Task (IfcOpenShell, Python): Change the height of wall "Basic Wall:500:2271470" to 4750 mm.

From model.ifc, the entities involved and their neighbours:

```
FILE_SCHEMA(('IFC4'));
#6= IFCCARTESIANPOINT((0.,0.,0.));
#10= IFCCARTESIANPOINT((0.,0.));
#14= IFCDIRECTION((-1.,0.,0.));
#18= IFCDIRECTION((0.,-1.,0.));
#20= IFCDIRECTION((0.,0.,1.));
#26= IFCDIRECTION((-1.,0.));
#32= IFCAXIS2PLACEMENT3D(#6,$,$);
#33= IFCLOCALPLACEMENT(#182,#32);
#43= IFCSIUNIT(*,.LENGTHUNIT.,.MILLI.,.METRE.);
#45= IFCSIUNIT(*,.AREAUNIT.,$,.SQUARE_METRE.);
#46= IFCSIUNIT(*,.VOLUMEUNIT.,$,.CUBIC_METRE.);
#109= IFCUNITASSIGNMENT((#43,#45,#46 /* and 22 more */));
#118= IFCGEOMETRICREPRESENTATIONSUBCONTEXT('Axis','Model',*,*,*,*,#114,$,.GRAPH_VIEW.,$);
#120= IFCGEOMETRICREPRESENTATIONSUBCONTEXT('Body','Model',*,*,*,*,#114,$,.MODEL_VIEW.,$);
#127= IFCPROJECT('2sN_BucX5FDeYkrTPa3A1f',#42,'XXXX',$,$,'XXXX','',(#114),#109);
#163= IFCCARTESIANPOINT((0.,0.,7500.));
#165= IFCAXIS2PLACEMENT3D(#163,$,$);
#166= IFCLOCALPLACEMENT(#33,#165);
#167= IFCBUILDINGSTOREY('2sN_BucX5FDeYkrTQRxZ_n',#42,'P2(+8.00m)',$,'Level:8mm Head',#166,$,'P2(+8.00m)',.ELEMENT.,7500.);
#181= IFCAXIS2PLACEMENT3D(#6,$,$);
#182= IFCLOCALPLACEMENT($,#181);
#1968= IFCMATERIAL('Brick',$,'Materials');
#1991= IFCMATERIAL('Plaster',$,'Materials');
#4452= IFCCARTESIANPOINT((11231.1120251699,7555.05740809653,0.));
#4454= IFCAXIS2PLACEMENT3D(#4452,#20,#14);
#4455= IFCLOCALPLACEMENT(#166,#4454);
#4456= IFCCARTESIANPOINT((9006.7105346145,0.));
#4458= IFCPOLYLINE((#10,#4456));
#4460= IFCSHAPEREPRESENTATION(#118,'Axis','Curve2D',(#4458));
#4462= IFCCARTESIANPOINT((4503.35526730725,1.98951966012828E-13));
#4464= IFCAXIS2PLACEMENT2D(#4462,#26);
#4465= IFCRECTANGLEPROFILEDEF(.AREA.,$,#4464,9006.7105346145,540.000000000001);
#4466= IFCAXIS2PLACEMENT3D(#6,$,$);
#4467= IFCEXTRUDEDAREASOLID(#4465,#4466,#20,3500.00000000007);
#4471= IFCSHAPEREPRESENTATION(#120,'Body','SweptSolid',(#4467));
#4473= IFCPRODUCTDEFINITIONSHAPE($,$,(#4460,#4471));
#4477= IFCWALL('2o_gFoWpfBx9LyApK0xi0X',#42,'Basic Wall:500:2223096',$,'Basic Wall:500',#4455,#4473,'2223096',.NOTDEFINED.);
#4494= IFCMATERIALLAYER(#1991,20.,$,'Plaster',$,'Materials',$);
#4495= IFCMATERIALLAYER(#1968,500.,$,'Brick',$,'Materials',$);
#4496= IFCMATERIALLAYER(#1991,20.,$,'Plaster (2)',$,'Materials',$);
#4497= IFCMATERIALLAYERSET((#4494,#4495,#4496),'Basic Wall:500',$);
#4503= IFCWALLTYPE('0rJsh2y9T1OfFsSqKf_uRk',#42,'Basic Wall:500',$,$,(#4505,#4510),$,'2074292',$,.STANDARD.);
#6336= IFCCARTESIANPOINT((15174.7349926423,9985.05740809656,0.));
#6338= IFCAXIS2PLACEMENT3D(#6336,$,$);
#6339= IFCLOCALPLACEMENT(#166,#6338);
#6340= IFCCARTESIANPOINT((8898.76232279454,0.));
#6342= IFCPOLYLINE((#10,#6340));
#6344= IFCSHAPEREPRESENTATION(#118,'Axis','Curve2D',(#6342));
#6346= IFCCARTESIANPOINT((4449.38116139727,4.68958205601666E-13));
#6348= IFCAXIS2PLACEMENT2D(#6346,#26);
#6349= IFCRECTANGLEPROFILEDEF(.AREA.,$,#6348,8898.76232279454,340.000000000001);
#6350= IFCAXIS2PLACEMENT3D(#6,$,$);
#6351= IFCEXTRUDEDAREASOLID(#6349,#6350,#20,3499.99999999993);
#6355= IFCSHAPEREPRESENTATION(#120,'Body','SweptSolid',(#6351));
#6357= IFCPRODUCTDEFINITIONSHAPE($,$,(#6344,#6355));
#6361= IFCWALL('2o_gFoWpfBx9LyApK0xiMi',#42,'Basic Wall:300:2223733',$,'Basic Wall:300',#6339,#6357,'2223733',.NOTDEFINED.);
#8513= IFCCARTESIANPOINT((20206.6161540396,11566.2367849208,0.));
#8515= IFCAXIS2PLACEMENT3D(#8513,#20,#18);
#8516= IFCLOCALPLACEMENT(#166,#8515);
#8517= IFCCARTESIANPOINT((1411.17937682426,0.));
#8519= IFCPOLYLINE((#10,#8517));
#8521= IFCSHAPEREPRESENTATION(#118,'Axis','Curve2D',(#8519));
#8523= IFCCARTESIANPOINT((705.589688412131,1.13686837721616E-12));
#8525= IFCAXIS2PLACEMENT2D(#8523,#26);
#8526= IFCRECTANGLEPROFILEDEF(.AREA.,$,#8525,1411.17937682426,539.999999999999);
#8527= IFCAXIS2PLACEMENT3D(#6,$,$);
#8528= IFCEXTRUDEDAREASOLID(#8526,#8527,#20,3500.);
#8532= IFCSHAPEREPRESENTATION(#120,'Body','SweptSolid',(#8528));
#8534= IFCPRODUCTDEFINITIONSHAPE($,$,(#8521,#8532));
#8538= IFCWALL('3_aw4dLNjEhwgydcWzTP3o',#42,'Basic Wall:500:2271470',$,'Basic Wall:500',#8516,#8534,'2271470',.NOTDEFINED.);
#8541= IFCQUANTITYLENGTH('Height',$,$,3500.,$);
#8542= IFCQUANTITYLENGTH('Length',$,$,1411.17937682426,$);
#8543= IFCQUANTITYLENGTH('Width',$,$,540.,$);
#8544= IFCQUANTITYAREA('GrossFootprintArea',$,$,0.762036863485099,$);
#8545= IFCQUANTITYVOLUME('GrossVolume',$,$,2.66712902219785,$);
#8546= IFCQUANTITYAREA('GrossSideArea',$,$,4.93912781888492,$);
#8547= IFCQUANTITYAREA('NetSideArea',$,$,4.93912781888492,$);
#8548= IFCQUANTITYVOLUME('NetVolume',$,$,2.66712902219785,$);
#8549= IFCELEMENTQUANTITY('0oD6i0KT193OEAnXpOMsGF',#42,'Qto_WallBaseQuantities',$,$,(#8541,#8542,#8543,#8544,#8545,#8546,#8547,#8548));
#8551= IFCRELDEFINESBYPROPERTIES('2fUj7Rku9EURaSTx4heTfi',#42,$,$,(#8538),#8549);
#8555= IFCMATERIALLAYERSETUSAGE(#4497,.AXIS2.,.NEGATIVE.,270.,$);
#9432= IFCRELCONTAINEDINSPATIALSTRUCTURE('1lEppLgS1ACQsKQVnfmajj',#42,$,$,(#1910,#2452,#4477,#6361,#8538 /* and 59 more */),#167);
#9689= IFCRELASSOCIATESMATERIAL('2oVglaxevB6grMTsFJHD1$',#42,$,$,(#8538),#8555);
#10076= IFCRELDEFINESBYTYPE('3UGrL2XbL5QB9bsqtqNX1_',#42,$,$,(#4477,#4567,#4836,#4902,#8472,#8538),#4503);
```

```python
import ifcopenshell
import ifcopenshell.api.pset
import ifcopenshell.geom
import ifcopenshell.util.element
import ifcopenshell.util.representation
import ifcopenshell.util.shape
import ifcopenshell.util.unit

model = ifcopenshell.open("model.ifc")
unit_scale = ifcopenshell.util.unit.calculate_unit_scale(model)
area_scale = ifcopenshell.util.unit.calculate_unit_scale(model, "AREAUNIT")
volume_scale = ifcopenshell.util.unit.calculate_unit_scale(model, "VOLUMEUNIT")
settings = ifcopenshell.geom.settings()


def volume(element):
    """Net volume in cubic metres, openings subtracted."""
    shape = ifcopenshell.geom.create_shape(settings, element)
    return ifcopenshell.util.shape.get_volume(shape.geometry)


wall = model.by_id(8538)
before = volume(wall)

body = ifcopenshell.util.representation.get_representation(wall, "Model", "Body")
solid = body.Items[0]
old_height = solid.Depth
solid.Depth = 4.75 / unit_scale
after = volume(wall)
thickness = 0.54  # wall thickness in metres

# Update the stored height, areas and volumes.
qto = model.by_id(ifcopenshell.util.element.get_pset(wall, "Qto_WallBaseQuantities", should_inherit=False)["id"])
ifcopenshell.api.pset.edit_qto(model, qto=qto, properties={
    "Height": solid.Depth,
    "GrossVolume": ifcopenshell.util.element.get_pset(wall, "Qto_WallBaseQuantities", "GrossVolume") * solid.Depth / old_height,
    "GrossSideArea": ifcopenshell.util.element.get_pset(wall, "Qto_WallBaseQuantities", "GrossSideArea") * solid.Depth / old_height,
    "NetSideArea": after / thickness / area_scale,
    "NetVolume": after / volume_scale,
})

print(f"height {old_height:g} -> {solid.Depth:g}, volume {before:.3f} -> {after:.3f} m3")

model.write("model_updated.ifc")
```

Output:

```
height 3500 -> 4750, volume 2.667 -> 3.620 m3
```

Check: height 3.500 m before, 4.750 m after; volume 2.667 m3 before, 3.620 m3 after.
